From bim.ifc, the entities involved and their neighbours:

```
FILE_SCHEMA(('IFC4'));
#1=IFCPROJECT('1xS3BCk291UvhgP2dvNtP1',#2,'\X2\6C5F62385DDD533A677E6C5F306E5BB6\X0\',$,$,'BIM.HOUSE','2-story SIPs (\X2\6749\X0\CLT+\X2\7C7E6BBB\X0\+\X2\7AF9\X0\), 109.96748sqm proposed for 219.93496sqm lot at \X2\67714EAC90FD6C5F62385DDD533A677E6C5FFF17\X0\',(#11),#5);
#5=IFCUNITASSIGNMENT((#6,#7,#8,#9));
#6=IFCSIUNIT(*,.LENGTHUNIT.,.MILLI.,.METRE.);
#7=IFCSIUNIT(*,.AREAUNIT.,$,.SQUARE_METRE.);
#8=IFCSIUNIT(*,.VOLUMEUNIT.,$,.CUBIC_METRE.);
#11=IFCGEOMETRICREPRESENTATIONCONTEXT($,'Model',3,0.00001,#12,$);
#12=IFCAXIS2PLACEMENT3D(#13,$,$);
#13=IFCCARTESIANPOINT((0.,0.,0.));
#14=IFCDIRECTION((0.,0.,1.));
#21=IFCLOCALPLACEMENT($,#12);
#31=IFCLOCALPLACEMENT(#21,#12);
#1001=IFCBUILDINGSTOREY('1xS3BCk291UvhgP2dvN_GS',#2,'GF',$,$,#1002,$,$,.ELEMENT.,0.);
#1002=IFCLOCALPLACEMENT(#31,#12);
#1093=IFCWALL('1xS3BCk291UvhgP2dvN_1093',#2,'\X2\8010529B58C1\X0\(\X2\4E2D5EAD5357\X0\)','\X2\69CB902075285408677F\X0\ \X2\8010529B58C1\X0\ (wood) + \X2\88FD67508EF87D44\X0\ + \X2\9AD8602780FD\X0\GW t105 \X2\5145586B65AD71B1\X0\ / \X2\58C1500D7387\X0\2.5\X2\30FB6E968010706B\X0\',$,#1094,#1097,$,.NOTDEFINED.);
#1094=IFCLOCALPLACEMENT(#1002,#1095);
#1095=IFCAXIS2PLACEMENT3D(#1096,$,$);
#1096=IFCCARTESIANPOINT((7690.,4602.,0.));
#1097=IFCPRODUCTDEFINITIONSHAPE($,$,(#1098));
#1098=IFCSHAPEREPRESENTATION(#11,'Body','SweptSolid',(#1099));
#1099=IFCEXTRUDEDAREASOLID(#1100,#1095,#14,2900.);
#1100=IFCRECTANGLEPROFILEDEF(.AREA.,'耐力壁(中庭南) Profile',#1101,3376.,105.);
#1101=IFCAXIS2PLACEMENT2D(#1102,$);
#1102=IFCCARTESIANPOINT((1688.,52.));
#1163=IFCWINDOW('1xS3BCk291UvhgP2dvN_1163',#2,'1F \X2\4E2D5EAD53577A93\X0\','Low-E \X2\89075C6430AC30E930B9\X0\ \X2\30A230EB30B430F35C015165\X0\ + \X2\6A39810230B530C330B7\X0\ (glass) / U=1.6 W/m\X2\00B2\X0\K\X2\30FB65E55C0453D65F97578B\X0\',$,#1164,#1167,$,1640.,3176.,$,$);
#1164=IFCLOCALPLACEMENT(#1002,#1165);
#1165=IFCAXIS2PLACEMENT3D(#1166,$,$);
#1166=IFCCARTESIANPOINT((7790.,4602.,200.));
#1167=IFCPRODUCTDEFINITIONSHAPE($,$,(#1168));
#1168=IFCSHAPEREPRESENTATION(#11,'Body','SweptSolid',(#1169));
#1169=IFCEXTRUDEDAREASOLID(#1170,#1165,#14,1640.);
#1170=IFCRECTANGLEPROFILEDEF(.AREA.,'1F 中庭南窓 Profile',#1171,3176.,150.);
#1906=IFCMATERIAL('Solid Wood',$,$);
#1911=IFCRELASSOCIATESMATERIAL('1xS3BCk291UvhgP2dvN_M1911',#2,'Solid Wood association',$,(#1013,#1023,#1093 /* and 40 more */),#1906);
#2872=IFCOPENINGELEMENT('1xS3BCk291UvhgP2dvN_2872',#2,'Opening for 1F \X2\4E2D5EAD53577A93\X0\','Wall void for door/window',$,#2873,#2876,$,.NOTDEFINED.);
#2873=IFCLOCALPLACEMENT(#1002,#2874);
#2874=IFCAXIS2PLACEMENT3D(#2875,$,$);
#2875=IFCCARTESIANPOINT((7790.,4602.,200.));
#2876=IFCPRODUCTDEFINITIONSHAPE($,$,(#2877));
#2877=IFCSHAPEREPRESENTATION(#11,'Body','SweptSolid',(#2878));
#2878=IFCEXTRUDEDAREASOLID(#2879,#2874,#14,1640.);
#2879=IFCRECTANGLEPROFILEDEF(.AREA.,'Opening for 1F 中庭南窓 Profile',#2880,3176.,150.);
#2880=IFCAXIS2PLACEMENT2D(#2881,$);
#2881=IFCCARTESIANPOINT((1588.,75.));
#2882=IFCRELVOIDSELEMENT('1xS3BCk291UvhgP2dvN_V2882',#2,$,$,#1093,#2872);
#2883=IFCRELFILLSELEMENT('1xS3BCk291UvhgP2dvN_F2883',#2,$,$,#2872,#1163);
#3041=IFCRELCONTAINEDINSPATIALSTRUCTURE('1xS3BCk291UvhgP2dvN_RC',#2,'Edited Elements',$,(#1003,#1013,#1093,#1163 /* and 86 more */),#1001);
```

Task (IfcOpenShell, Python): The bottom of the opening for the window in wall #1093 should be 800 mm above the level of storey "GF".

```python
import numpy as np
import ifcopenshell
import ifcopenshell.api.geometry
import ifcopenshell.geom
import ifcopenshell.util.element
import ifcopenshell.util.placement
import ifcopenshell.util.shape
import ifcopenshell.util.unit

model = ifcopenshell.open("bim.ifc")
unit_scale = ifcopenshell.util.unit.calculate_unit_scale(model)

window = model.by_id(1163)
opening = window.FillsVoids[0].RelatingOpeningElement
storey = ifcopenshell.util.element.get_container(window, ifc_class="IfcBuildingStorey")
level = ifcopenshell.util.placement.get_local_placement(storey.ObjectPlacement)[2, 3]

# The opening's origin need not be at the sill, so measure its lowest point.
shape = ifcopenshell.geom.create_shape(ifcopenshell.geom.settings(), opening)
bottom = ifcopenshell.util.shape.get_shape_bottom_elevation(shape, shape.geometry) / unit_scale
dz = level + 800.0 - bottom

shift = np.array([0.0, 0.0, dz])
# The window is not placed relative to its opening, so move both.
for product in (opening, window):
    matrix = ifcopenshell.util.placement.get_local_placement(product.ObjectPlacement)
    matrix[:3, 3] += shift
    ifcopenshell.api.geometry.edit_object_placement(model, product=product, matrix=matrix, is_si=False)

print(f"moved by {dz * unit_scale:+.3f} m")

model.write("bim_rev.ifc")
```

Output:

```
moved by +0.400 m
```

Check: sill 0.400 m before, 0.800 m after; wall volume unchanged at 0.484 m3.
